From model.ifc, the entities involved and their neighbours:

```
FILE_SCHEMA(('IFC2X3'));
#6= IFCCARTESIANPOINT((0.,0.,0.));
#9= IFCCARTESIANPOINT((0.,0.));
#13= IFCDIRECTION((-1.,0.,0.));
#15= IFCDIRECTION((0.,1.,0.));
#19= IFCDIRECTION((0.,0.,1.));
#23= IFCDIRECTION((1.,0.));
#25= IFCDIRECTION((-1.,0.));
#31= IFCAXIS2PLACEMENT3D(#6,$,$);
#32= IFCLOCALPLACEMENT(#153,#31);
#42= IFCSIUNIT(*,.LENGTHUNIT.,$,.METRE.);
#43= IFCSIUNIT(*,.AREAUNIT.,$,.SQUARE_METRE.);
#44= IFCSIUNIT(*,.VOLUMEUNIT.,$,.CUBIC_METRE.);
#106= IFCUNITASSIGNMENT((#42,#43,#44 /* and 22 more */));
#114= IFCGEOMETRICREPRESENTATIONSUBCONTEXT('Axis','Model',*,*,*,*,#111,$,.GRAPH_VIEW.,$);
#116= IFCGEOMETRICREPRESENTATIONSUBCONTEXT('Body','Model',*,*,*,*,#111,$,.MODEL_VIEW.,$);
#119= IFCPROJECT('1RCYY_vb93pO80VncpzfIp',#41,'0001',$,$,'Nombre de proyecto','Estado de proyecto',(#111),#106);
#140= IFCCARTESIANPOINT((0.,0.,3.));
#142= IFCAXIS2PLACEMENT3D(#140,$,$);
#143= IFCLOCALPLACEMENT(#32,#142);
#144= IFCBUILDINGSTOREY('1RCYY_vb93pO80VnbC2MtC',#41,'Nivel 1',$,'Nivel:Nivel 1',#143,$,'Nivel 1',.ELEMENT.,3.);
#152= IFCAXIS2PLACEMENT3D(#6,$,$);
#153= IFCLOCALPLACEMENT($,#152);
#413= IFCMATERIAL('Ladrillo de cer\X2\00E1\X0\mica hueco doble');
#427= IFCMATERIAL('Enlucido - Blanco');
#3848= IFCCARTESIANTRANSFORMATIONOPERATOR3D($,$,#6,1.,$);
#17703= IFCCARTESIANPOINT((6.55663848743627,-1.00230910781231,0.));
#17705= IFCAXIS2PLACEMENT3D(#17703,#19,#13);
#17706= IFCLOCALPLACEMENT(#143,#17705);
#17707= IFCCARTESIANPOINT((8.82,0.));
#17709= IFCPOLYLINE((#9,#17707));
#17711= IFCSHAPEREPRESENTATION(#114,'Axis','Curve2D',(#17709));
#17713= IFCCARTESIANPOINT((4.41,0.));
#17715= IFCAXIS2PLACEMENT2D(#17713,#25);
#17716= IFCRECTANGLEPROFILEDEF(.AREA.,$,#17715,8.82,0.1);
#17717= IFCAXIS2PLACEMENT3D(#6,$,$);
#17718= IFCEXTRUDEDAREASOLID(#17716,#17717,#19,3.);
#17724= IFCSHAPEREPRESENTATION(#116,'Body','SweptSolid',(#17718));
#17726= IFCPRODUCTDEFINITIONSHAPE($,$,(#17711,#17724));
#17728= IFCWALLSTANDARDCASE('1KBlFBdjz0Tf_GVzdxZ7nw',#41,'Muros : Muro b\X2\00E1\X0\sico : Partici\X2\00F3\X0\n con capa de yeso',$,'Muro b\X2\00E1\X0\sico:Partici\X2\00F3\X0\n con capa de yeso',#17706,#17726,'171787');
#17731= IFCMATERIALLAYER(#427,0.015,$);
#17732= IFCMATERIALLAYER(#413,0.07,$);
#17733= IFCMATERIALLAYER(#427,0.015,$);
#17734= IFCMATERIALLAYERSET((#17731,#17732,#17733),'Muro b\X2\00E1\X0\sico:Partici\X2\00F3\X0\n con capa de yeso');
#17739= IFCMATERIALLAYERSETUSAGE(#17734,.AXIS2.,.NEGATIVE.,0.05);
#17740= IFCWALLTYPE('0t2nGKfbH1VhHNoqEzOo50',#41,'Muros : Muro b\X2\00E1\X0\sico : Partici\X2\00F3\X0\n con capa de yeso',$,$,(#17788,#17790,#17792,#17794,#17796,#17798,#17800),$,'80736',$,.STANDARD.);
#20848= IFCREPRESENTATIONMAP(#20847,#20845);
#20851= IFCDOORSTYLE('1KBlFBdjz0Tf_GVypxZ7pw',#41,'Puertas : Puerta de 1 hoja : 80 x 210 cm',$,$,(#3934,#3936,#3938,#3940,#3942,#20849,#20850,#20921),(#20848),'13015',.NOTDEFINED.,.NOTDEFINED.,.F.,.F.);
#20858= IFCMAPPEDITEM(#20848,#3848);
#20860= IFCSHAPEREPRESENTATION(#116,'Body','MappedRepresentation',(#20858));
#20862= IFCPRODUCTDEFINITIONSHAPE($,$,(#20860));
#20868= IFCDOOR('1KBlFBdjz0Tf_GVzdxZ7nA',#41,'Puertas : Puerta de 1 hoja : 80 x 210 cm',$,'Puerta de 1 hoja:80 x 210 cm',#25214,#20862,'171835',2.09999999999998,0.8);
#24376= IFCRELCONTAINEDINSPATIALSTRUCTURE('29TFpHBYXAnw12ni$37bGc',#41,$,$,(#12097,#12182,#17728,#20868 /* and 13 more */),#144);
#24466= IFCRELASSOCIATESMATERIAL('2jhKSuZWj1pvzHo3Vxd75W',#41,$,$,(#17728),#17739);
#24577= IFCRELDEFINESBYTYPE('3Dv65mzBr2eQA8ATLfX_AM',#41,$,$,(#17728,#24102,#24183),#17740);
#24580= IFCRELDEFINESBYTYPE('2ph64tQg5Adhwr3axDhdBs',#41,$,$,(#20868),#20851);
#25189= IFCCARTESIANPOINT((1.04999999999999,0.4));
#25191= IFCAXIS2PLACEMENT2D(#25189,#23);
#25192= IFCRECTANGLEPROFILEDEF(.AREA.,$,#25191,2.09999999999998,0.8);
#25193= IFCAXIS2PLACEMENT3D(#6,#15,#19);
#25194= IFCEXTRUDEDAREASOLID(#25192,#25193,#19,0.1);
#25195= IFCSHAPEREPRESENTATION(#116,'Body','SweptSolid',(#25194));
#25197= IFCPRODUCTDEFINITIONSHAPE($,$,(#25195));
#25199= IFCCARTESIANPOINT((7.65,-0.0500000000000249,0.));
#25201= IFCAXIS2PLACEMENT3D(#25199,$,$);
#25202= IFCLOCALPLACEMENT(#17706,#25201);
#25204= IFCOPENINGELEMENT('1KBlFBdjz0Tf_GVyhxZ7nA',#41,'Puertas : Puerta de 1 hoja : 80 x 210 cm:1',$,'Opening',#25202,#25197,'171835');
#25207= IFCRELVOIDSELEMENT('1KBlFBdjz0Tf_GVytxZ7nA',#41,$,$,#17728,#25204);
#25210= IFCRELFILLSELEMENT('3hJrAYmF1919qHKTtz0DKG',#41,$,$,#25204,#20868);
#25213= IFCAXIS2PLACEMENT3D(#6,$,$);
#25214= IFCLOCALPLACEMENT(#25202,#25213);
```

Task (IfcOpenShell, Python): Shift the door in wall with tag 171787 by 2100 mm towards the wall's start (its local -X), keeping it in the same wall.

```python
import ifcopenshell
import ifcopenshell.api.geometry
import ifcopenshell.util.placement
import ifcopenshell.util.unit

model = ifcopenshell.open("model.ifc")
unit_scale = ifcopenshell.util.unit.calculate_unit_scale(model)

door = model.by_guid("1KBlFBdjz0Tf_GVzdxZ7nA")
opening = door.FillsVoids[0].RelatingOpeningElement
wall = opening.VoidsElements[0].RelatingBuildingElement

wall_matrix = ifcopenshell.util.placement.get_local_placement(wall.ObjectPlacement)
shift = wall_matrix[:3, 0] * -2.1 / unit_scale
before = ifcopenshell.util.placement.get_local_placement(door.ObjectPlacement)[:3, 3].copy()

# The door is placed relative to its opening, so it follows when the opening moves.
matrix = ifcopenshell.util.placement.get_local_placement(opening.ObjectPlacement)
matrix[:3, 3] += shift
ifcopenshell.api.geometry.edit_object_placement(
    model, product=opening, matrix=matrix, is_si=False, should_transform_children=True
)

after = ifcopenshell.util.placement.get_local_placement(door.ObjectPlacement)[:3, 3]
print("door moved by", (after - before).round(3) + 0.0)

model.write("model_edited.ifc")
```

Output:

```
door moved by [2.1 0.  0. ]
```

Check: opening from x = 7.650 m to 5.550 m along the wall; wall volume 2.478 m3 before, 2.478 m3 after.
